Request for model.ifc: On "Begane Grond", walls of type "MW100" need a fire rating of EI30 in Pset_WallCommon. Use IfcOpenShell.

First a look at what the model holds.

```python
import ifcopenshell
import ifcopenshell.util.element

model = ifcopenshell.open("model.ifc")
print(model.schema)
storey = next(s for s in model.by_type("IfcBuildingStorey") if s.Name == "Begane Grond")
walls = [e for e in ifcopenshell.util.element.get_decomposition(storey) if e.is_a("IfcWall")]
seen = {}
for e in walls:
    element_type = ifcopenshell.util.element.get_type(e)
    key = (element_type.Name if element_type != e and element_type else None, ifcopenshell.util.element.get_pset(e, "Pset_WallCommon", "FireRating"))
    seen[key] = seen.get(key, 0) + 1
for (name, value), count in sorted(seen.items(), key=str):
    print(count, "x", name, "|", value)
```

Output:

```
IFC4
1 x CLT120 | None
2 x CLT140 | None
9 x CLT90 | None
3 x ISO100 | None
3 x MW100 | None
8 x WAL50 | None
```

```python
import ifcopenshell
import ifcopenshell.api.pset
import ifcopenshell.util.element

model = ifcopenshell.open("model.ifc")

storey = next(s for s in model.by_type("IfcBuildingStorey") if s.Name == "Begane Grond")
walls = [e for e in ifcopenshell.util.element.get_decomposition(storey) if e.is_a("IfcWall")]

count = 0
for e in walls:
    element_type = ifcopenshell.util.element.get_type(e)
    if element_type in (None, e) or element_type.Name != "MW100":
        continue
    # add_pset returns the element's existing set when there is one.
    pset = ifcopenshell.api.pset.add_pset(model, product=e, name="Pset_WallCommon")
    ifcopenshell.api.pset.edit_pset(model, pset=pset, properties={"FireRating": "EI30"})
    count += 1

print(count, "walls updated")

model.write("model-out.ifc")
```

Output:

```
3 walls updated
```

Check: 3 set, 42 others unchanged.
